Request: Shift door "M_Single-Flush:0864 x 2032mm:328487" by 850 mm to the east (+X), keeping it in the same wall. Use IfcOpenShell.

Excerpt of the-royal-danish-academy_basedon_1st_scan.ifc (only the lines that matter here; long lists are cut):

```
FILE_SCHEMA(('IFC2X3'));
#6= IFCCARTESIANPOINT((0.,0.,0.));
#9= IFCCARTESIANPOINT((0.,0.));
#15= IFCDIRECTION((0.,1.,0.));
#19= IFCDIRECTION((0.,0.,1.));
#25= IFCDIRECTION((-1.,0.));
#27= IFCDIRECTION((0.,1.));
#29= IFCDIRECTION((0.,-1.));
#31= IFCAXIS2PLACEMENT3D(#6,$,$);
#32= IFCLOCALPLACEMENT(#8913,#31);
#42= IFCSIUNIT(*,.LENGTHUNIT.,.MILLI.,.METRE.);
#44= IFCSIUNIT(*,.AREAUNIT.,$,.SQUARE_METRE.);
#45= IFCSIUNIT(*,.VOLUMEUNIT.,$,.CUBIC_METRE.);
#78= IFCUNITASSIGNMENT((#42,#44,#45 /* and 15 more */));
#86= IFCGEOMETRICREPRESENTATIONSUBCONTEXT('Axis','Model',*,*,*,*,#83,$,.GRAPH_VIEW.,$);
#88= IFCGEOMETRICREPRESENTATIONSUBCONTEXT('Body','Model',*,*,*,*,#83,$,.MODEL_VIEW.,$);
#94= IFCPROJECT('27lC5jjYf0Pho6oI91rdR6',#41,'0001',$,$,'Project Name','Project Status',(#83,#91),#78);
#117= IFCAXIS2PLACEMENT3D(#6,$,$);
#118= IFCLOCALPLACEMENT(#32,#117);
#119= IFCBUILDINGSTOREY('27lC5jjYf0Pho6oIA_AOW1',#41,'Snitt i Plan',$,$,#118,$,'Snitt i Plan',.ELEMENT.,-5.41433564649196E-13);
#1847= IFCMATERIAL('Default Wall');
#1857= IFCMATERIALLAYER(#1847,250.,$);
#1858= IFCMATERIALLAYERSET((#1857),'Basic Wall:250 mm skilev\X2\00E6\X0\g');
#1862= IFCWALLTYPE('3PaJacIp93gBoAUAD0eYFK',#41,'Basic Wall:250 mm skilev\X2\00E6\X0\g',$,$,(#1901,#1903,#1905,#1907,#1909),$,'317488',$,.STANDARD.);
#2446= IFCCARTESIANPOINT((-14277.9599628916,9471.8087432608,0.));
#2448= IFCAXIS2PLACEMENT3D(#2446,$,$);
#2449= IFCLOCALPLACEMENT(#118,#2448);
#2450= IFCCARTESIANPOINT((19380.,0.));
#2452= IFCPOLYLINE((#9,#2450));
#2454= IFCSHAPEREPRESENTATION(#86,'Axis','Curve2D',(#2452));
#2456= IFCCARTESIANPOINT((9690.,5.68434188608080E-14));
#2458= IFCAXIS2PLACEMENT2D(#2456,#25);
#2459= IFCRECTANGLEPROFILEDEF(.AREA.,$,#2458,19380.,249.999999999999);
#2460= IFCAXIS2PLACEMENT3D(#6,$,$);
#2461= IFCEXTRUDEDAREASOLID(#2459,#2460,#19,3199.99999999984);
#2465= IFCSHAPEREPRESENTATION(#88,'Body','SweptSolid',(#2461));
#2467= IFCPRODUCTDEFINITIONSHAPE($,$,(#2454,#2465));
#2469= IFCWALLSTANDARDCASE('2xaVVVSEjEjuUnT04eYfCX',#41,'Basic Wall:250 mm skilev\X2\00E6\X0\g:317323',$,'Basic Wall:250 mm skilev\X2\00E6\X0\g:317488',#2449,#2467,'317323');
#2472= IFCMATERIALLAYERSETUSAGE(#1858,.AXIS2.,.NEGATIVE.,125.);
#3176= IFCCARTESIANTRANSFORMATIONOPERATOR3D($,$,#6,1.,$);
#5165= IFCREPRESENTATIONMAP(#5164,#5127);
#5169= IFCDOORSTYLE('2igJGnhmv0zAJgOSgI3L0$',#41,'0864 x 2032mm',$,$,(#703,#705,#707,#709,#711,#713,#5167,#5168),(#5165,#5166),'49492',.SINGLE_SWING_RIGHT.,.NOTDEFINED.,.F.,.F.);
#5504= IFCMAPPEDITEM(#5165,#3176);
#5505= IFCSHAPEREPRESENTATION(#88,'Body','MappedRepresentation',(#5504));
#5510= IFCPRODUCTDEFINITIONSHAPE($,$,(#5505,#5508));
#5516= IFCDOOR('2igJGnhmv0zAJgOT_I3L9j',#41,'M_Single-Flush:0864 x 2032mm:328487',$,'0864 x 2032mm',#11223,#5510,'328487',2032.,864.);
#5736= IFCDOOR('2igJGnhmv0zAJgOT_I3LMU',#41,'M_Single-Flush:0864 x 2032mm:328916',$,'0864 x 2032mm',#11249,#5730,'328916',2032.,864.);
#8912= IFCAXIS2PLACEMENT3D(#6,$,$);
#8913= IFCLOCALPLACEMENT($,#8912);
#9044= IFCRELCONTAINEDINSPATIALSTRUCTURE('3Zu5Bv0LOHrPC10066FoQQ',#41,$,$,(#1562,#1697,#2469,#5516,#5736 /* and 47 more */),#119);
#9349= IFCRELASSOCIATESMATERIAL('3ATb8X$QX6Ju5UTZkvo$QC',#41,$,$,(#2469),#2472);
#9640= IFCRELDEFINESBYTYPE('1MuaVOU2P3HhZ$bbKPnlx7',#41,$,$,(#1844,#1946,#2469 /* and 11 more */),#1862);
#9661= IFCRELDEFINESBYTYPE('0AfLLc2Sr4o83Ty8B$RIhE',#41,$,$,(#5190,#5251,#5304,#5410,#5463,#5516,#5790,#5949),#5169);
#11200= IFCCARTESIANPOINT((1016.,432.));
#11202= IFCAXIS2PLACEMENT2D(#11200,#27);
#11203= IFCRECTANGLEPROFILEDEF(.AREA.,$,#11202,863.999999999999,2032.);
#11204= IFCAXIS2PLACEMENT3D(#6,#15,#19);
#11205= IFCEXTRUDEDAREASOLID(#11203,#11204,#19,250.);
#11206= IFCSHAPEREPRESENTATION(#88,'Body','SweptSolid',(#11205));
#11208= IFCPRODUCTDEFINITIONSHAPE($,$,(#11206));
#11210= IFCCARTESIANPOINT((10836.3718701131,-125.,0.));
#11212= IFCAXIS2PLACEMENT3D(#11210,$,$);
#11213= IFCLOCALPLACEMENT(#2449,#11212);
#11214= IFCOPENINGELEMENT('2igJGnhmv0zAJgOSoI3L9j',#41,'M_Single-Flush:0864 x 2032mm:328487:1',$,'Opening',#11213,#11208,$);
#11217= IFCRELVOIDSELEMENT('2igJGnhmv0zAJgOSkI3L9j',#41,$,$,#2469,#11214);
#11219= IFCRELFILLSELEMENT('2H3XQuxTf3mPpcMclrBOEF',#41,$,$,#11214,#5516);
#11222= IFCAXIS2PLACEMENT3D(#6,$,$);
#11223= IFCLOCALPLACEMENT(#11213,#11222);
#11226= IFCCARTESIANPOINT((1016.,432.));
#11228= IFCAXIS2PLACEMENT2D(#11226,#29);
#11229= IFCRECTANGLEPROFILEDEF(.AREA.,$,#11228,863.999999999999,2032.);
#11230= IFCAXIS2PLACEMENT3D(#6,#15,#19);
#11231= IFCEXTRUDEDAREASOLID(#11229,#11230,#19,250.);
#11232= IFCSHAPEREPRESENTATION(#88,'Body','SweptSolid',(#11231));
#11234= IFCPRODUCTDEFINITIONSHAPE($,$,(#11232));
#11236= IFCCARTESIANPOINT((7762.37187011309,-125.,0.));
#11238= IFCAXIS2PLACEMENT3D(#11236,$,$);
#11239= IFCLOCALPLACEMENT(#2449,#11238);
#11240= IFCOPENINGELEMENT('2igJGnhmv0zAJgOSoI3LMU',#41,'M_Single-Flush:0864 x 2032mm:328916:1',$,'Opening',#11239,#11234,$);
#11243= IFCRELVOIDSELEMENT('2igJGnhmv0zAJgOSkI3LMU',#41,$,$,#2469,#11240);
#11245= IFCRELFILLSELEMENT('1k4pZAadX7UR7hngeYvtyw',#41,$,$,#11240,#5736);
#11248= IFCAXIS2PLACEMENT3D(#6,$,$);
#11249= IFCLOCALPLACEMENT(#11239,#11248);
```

```python
import ifcopenshell
import ifcopenshell.api.geometry
import ifcopenshell.util.placement

model = ifcopenshell.open("the-royal-danish-academy_basedon_1st_scan.ifc")

door = model.by_guid("2igJGnhmv0zAJgOT_I3L9j")
opening = door.FillsVoids[0].RelatingOpeningElement
wall = opening.VoidsElements[0].RelatingBuildingElement

wall_matrix = ifcopenshell.util.placement.get_local_placement(wall.ObjectPlacement)
shift = wall_matrix[:3, 0] * 850.0
before = ifcopenshell.util.placement.get_local_placement(door.ObjectPlacement)[:3, 3].copy()

# The door is placed relative to its opening, so it follows when the opening moves.
matrix = ifcopenshell.util.placement.get_local_placement(opening.ObjectPlacement)
matrix[:3, 3] += shift
ifcopenshell.api.geometry.edit_object_placement(
    model, product=opening, matrix=matrix, is_si=False, should_transform_children=True
)

after = ifcopenshell.util.placement.get_local_placement(door.ObjectPlacement)[:3, 3]
print("door moved by", (after - before).round(3) + 0.0)

model.write("the-royal-danish-academy_basedon_1st_scan_edited.ifc")
```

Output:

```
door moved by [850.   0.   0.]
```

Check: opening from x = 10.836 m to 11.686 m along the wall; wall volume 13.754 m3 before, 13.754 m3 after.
